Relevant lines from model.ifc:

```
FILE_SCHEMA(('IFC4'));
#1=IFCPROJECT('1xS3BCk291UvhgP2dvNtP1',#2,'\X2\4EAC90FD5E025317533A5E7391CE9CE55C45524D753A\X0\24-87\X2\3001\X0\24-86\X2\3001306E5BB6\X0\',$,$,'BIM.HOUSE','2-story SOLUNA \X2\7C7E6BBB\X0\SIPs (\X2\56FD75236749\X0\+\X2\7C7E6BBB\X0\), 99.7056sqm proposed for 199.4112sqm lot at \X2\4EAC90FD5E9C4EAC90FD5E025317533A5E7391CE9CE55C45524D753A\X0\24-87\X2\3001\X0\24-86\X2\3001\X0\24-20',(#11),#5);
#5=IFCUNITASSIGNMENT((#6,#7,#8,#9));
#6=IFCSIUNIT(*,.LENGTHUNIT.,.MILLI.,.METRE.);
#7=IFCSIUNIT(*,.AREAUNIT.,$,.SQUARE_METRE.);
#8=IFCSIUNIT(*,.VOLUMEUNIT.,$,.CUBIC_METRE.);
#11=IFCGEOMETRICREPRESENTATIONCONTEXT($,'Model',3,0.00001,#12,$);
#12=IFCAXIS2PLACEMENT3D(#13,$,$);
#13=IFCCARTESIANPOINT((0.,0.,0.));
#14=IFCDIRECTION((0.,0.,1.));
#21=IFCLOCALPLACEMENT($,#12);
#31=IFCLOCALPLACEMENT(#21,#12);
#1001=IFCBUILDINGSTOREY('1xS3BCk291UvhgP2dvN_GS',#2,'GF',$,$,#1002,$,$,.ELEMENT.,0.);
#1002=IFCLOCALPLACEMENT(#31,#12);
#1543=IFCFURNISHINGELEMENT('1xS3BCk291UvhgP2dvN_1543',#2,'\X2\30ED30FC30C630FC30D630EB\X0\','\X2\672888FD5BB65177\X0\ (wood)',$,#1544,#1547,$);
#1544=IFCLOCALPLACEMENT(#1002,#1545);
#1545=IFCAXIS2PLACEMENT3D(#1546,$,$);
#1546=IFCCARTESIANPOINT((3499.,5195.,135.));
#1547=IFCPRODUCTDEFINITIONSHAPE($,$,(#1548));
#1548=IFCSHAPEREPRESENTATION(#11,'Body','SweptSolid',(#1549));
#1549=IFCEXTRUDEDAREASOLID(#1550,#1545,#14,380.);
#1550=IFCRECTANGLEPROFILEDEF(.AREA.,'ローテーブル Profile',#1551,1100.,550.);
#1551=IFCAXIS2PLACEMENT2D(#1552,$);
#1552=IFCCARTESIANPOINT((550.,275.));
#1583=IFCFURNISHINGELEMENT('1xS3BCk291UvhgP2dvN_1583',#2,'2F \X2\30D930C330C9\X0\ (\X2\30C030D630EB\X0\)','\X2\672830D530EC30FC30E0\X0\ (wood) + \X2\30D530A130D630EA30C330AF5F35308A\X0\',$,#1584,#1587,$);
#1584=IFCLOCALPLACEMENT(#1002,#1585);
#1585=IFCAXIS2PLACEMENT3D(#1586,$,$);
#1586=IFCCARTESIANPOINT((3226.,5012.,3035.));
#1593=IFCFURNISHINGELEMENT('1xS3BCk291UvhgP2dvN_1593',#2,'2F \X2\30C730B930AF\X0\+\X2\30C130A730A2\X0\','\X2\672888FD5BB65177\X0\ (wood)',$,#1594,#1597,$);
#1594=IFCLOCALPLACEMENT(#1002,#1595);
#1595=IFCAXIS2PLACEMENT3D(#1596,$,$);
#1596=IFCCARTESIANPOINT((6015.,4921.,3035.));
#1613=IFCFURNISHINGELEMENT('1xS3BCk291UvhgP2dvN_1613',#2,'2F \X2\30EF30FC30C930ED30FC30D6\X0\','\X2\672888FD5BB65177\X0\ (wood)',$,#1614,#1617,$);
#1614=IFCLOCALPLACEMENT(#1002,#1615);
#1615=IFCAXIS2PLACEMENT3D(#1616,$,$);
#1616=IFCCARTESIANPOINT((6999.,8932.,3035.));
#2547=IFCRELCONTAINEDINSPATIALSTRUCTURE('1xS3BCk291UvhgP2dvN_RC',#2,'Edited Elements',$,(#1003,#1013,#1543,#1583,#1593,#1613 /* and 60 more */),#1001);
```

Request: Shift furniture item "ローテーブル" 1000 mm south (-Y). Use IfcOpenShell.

```python
import ifcopenshell
import ifcopenshell.api.geometry
import ifcopenshell.util.placement
import ifcopenshell.util.unit

model = ifcopenshell.open("model.ifc")
unit_scale = ifcopenshell.util.unit.calculate_unit_scale(model)

item = model.by_guid("1xS3BCk291UvhgP2dvN_1543")
matrix = ifcopenshell.util.placement.get_local_placement(item.ObjectPlacement)
matrix[1, 3] -= 1 / unit_scale
ifcopenshell.api.geometry.edit_object_placement(model, product=item, matrix=matrix, is_si=False)

print(ifcopenshell.util.placement.get_local_placement(item.ObjectPlacement).round(3) + 0.0)

model.write("model_edited.ifc")
```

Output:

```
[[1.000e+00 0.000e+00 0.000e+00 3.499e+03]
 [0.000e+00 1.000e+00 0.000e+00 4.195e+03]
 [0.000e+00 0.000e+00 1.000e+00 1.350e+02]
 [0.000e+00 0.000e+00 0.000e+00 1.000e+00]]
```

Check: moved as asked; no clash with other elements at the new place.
